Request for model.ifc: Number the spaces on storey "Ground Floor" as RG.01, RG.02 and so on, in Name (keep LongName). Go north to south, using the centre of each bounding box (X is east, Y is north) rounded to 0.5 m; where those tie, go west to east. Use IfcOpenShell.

First a look at what the model holds.

```python
import ifcopenshell
import ifcopenshell.util.element
import ifcopenshell.util.placement

model = ifcopenshell.open("model.ifc")
print(model.schema)
storey = next(s for s in model.by_type("IfcBuildingStorey") if s.Name == "Ground Floor")
spaces = [e for e in ifcopenshell.util.element.get_decomposition(storey) if e.is_a("IfcSpace")]
for e in sorted(spaces, key=lambda e: e.id()):
    origin = ifcopenshell.util.placement.get_local_placement(e.ObjectPlacement)[:3, 3]
    print(e.id(), e.Name, e.LongName, origin.round(2) + 0.0, sep=" | ")
```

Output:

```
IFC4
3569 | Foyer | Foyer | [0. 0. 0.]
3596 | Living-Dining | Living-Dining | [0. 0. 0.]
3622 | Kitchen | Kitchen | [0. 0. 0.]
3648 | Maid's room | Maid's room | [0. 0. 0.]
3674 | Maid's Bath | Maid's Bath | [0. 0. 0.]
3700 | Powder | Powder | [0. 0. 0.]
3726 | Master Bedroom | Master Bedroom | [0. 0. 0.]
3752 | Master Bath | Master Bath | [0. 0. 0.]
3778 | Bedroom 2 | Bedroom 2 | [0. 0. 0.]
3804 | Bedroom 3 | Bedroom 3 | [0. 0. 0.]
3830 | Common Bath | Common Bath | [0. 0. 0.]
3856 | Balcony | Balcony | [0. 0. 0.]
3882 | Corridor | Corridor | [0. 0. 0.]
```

```python
import ifcopenshell
import ifcopenshell.geom
import ifcopenshell.util.element
import ifcopenshell.util.shape

model = ifcopenshell.open("model.ifc")
settings = ifcopenshell.geom.settings()
settings.set("use-world-coords", True)


def centre(element):
    shape = ifcopenshell.geom.create_shape(settings, element)
    return ifcopenshell.util.shape.get_bbox_centroid(shape.geometry)


storey = next(s for s in model.by_type("IfcBuildingStorey") if s.Name == "Ground Floor")
spaces = [e for e in ifcopenshell.util.element.get_decomposition(storey) if e.is_a("IfcSpace")]

# Insertion points can sit at a corner or the storey origin, so sort by the geometry (in metres).
centres = {e: centre(e) for e in spaces}
spaces.sort(key=lambda e: (-round(centres[e][1] / 0.5), centres[e][0]))

for i, e in enumerate(spaces, start=1):
    number = f"RG.{i:02d}"
    e.Name = number
    print(e.id(), number)

model.write("model-out.ifc")
```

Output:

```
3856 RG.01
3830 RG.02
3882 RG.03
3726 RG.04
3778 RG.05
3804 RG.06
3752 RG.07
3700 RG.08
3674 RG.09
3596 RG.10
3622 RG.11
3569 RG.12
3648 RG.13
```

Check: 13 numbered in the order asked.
